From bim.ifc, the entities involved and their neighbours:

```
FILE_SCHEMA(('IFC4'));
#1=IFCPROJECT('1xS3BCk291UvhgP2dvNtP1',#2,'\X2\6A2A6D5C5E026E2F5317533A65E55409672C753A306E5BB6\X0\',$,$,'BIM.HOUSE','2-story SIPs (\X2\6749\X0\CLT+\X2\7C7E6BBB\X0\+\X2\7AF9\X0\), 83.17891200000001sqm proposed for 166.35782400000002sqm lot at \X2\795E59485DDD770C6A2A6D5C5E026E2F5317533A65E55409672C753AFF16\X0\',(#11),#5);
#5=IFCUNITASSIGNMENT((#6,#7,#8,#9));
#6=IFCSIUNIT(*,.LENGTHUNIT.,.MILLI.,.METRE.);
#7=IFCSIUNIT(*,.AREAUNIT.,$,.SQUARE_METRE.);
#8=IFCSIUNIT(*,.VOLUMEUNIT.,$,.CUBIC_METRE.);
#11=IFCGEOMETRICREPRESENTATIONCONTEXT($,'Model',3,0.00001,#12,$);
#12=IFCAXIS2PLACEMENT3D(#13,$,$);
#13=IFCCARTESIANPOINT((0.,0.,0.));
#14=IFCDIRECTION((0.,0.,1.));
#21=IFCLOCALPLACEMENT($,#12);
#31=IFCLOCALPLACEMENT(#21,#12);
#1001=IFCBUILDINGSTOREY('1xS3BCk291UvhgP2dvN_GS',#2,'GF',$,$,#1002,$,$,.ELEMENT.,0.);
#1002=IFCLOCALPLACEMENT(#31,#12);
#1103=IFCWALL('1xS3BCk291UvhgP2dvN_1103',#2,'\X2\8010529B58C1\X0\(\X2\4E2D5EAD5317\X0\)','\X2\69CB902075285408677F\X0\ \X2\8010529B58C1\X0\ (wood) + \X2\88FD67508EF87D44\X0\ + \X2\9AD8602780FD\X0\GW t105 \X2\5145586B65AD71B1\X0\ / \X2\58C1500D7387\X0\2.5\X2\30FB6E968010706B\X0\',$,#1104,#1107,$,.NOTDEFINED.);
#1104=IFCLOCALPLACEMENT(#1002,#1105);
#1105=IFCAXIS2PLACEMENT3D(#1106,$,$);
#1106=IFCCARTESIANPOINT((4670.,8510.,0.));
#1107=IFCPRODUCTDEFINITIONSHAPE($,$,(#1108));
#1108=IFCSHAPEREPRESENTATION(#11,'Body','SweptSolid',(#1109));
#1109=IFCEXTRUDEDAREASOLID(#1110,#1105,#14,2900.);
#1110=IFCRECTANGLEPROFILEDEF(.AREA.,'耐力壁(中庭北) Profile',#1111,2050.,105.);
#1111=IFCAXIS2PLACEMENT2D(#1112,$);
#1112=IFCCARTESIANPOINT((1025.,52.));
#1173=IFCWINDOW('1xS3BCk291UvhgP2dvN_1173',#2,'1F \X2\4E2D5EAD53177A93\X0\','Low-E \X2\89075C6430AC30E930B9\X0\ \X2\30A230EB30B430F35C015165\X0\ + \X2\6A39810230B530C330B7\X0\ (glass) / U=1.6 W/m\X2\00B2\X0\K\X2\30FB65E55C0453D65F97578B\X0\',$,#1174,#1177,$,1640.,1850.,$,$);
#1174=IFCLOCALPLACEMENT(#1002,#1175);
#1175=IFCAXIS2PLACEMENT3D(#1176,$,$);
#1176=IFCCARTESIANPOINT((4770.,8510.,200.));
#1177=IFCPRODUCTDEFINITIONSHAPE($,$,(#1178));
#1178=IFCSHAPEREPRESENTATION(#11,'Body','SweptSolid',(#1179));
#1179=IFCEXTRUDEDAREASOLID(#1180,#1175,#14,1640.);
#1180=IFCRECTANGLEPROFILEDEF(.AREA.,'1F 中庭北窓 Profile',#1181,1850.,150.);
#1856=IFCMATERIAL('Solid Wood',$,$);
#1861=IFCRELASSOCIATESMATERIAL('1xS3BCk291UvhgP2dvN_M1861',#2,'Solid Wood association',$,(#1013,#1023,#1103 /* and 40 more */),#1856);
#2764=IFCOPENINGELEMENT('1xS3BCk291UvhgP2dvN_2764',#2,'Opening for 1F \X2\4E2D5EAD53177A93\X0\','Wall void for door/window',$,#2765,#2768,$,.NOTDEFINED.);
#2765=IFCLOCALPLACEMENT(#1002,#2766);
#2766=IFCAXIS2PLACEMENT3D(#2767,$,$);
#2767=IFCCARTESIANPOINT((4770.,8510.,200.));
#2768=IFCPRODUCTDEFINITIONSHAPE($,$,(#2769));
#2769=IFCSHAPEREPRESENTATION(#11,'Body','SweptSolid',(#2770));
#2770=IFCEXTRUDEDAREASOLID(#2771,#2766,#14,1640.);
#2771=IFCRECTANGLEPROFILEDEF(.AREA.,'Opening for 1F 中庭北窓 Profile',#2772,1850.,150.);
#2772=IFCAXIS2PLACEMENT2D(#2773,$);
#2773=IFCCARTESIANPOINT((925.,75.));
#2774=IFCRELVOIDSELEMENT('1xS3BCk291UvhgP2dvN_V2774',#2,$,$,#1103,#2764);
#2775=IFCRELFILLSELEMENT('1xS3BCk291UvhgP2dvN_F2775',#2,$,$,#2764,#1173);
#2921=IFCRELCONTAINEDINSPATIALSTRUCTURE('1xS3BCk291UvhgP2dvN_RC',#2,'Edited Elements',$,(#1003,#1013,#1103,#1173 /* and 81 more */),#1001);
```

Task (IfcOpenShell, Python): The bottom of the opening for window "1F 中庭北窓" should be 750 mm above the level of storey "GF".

```python
import numpy as np
import ifcopenshell
import ifcopenshell.api.geometry
import ifcopenshell.geom
import ifcopenshell.util.element
import ifcopenshell.util.placement
import ifcopenshell.util.shape
import ifcopenshell.util.unit

model = ifcopenshell.open("bim.ifc")
unit_scale = ifcopenshell.util.unit.calculate_unit_scale(model)

window = model.by_id(1173)
opening = window.FillsVoids[0].RelatingOpeningElement
storey = ifcopenshell.util.element.get_container(window, ifc_class="IfcBuildingStorey")
level = ifcopenshell.util.placement.get_local_placement(storey.ObjectPlacement)[2, 3]

# The opening's origin need not be at the sill, so measure its lowest point.
shape = ifcopenshell.geom.create_shape(ifcopenshell.geom.settings(), opening)
bottom = ifcopenshell.util.shape.get_shape_bottom_elevation(shape, shape.geometry) / unit_scale
dz = level + 750.0 - bottom

shift = np.array([0.0, 0.0, dz])
# The window is not placed relative to its opening, so move both.
for product in (opening, window):
    matrix = ifcopenshell.util.placement.get_local_placement(product.ObjectPlacement)
    matrix[:3, 3] += shift
    ifcopenshell.api.geometry.edit_object_placement(model, product=product, matrix=matrix, is_si=False)

print(f"moved by {dz * unit_scale:+.3f} m")

model.write("bim_v2.ifc")
```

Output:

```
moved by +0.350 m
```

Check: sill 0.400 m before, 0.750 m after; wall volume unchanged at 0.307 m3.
